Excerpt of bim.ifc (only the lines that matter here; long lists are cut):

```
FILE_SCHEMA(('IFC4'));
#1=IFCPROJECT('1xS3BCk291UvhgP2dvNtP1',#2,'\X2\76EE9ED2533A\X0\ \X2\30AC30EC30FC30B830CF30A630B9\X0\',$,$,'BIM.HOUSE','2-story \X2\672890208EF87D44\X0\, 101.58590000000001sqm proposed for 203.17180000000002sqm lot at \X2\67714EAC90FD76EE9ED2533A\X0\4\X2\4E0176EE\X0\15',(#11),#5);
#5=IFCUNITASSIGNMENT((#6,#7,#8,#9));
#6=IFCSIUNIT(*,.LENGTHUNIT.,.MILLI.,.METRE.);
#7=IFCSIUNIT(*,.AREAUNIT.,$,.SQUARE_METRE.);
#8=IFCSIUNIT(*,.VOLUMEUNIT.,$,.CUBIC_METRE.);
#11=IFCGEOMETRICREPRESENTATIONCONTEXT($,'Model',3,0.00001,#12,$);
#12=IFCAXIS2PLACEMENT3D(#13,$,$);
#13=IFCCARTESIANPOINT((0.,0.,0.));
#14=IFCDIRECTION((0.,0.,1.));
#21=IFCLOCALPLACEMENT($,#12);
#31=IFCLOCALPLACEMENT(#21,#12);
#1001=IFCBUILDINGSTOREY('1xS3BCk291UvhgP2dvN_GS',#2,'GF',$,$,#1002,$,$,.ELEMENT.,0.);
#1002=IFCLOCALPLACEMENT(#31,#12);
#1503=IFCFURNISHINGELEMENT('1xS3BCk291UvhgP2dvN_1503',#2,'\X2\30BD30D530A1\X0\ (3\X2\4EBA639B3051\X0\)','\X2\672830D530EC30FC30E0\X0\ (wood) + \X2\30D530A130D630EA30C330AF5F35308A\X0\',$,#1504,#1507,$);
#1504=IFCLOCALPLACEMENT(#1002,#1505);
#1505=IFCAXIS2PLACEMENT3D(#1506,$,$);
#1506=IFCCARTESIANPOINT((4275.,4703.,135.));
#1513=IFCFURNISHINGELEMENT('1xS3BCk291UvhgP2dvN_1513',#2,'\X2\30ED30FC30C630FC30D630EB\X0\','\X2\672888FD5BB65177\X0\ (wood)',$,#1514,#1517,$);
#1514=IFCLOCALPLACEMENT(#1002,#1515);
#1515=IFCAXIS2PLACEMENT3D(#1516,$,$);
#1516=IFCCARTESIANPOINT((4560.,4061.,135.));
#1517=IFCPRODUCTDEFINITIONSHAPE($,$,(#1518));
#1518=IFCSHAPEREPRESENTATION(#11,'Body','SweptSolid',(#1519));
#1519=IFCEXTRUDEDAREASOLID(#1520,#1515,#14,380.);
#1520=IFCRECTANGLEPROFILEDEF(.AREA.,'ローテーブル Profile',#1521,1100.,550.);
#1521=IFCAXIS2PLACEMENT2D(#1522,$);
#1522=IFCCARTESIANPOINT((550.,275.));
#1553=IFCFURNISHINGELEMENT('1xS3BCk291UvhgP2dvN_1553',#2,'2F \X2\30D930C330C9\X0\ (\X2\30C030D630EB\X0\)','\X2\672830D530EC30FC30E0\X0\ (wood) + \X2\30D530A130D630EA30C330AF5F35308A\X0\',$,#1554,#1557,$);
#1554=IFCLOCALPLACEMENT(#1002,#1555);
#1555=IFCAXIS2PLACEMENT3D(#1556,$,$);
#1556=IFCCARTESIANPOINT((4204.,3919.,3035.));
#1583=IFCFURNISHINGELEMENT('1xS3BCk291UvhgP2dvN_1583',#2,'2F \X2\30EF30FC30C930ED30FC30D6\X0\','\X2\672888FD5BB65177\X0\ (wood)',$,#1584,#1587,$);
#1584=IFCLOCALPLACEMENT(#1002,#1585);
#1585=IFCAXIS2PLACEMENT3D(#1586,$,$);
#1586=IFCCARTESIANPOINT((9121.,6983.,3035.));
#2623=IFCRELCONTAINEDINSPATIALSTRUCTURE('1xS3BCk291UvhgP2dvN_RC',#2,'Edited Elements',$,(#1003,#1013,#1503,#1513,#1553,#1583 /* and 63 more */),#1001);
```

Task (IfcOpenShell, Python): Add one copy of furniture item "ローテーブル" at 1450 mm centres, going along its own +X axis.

```python
import ifcopenshell
import ifcopenshell.api.geometry
import ifcopenshell.api.root
import ifcopenshell.util.element
import ifcopenshell.util.placement
import ifcopenshell.util.unit

model = ifcopenshell.open("bim.ifc")
unit_scale = ifcopenshell.util.unit.calculate_unit_scale(model)


def reuse_history(source, copy):
    """copy_class also copies each property set's owner history, people and application; keep the originals."""
    for rel in copy.IsDefinedBy:
        if rel.is_a("IfcRelDefinesByProperties") and (history := rel.RelatingPropertyDefinition.OwnerHistory):
            rel.RelatingPropertyDefinition.OwnerHistory = source.OwnerHistory
            ifcopenshell.util.element.remove_deep2(model, history)


source = model.by_guid("1xS3BCk291UvhgP2dvN_1513")
base = ifcopenshell.util.placement.get_local_placement(source.ObjectPlacement)
step = base[:3, 0] * 1.45 / unit_scale

for i in range(1, 2):
    copy = ifcopenshell.api.root.copy_class(model, product=source)
    copy.Representation = ifcopenshell.util.element.copy_deep(
        model, source.Representation, exclude=["IfcGeometricRepresentationContext", "IfcRepresentationMap"]
    )
    reuse_history(source, copy)
    matrix = base.copy()
    matrix[:3, 3] += i * step
    print("added at", matrix[:3, 3].round(3) + 0.0)
    ifcopenshell.api.geometry.edit_object_placement(model, product=copy, matrix=matrix, is_si=False)

model.write("bim_v2.ifc")
```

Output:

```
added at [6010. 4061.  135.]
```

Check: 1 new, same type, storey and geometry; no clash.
